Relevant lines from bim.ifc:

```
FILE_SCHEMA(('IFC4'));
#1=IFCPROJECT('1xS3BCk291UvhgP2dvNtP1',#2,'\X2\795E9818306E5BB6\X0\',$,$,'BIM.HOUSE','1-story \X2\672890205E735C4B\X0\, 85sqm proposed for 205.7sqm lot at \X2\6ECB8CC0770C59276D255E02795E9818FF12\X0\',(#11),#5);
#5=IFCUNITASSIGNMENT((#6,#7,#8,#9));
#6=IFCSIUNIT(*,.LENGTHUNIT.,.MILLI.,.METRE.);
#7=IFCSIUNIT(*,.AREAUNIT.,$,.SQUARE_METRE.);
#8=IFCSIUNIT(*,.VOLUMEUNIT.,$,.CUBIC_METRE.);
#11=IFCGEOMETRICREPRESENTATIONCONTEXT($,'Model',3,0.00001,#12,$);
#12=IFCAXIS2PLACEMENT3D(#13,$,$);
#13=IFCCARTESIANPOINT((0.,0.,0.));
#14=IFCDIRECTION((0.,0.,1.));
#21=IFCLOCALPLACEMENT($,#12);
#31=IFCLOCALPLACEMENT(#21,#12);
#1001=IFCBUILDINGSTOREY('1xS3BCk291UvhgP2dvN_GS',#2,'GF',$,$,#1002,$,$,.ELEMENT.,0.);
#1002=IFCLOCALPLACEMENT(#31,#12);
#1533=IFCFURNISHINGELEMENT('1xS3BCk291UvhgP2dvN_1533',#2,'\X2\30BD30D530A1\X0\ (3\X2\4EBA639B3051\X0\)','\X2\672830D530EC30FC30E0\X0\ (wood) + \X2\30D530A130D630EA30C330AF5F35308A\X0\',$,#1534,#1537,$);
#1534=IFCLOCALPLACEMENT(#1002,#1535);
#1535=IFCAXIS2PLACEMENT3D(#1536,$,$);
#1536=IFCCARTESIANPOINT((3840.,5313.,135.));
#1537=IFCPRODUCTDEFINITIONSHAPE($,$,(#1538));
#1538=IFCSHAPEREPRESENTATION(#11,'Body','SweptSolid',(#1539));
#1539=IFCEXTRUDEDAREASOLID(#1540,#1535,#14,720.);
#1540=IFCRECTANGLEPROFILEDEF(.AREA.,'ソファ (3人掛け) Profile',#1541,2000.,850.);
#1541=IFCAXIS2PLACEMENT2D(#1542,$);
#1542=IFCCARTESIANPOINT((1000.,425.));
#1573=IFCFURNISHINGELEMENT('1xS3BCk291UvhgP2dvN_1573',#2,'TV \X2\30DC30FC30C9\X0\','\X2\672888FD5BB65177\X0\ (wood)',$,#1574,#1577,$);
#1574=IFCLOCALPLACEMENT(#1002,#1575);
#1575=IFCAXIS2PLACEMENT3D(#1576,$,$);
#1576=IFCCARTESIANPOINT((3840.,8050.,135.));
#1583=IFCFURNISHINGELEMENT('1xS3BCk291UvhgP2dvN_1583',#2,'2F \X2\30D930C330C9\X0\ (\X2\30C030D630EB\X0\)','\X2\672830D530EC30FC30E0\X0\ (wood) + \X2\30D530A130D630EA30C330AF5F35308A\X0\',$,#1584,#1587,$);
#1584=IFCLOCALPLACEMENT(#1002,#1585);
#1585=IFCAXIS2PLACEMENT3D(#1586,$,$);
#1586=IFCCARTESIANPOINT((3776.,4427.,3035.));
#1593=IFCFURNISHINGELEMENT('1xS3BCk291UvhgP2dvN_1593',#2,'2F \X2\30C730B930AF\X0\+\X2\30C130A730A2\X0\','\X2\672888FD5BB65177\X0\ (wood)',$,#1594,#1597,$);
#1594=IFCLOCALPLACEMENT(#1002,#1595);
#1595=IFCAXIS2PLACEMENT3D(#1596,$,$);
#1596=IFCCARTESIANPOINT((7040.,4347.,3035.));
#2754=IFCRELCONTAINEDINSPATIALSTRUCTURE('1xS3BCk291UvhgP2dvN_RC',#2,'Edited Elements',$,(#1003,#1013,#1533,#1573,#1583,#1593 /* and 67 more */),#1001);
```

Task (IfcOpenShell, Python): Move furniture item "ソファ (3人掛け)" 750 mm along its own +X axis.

```python
import ifcopenshell
import ifcopenshell.api.geometry
import ifcopenshell.util.placement
import ifcopenshell.util.unit

model = ifcopenshell.open("bim.ifc")
unit_scale = ifcopenshell.util.unit.calculate_unit_scale(model)

item = model.by_id(1533)
matrix = ifcopenshell.util.placement.get_local_placement(item.ObjectPlacement)
matrix[:3, 3] += matrix[:3, 0] * 0.75 / unit_scale
ifcopenshell.api.geometry.edit_object_placement(model, product=item, matrix=matrix, is_si=False)

print(ifcopenshell.util.placement.get_local_placement(item.ObjectPlacement).round(3) + 0.0)

model.write("bim_v2.ifc")
```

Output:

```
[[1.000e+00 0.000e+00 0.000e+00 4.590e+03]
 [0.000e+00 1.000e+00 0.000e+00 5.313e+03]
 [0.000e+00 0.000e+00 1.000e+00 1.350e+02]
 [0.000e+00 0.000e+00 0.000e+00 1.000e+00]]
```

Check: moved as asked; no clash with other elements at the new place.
